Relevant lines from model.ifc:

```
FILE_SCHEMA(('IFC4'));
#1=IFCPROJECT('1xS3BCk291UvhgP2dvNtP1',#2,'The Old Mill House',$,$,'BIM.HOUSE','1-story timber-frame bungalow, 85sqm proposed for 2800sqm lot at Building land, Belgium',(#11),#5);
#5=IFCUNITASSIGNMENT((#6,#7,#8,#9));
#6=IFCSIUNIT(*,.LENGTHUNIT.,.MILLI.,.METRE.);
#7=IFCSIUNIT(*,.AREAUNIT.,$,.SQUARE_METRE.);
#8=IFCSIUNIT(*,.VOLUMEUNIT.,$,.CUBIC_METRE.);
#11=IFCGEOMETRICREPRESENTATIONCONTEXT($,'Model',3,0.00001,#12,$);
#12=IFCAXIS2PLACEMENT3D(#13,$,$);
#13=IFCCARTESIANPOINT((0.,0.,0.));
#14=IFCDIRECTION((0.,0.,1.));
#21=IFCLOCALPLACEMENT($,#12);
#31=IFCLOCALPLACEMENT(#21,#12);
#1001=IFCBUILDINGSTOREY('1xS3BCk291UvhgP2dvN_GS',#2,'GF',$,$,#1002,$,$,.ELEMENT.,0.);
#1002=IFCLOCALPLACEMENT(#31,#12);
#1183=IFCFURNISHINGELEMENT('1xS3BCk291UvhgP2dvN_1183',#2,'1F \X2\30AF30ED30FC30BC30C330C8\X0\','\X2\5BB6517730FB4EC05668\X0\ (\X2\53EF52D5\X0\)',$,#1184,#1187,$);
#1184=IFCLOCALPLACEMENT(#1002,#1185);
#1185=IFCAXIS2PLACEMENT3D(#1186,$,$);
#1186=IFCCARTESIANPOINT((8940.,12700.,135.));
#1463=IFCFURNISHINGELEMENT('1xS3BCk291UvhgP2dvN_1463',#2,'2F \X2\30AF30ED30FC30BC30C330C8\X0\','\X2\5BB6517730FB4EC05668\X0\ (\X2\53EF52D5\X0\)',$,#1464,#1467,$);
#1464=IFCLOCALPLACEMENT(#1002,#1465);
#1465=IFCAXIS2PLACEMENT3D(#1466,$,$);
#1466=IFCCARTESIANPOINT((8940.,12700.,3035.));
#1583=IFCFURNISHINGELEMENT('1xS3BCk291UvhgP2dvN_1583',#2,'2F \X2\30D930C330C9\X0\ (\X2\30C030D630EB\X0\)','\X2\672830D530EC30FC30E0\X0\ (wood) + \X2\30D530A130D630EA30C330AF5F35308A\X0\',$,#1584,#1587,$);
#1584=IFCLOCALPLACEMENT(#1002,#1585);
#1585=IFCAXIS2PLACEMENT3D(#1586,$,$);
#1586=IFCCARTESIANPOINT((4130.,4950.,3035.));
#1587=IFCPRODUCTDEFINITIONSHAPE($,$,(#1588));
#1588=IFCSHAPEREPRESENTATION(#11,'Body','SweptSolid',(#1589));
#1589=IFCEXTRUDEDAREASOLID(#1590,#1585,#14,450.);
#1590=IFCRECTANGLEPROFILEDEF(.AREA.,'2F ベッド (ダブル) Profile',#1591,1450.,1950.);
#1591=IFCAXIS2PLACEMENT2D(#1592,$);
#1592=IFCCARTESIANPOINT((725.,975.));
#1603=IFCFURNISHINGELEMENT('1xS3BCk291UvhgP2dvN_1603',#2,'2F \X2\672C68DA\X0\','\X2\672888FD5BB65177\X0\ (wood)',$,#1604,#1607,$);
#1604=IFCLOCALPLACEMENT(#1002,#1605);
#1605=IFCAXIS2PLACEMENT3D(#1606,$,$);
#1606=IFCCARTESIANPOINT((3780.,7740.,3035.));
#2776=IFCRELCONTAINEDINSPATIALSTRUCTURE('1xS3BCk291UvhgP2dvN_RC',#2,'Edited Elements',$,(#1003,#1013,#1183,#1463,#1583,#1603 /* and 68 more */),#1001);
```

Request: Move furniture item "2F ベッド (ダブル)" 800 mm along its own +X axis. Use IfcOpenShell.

```python
import ifcopenshell
import ifcopenshell.api.geometry
import ifcopenshell.util.placement

model = ifcopenshell.open("model.ifc")

item = model.by_id(1583)
matrix = ifcopenshell.util.placement.get_local_placement(item.ObjectPlacement)
matrix[:3, 3] += matrix[:3, 0] * 800.0
ifcopenshell.api.geometry.edit_object_placement(model, product=item, matrix=matrix, is_si=False)

print(ifcopenshell.util.placement.get_local_placement(item.ObjectPlacement).round(3) + 0.0)

model.write("model_updated.ifc")
```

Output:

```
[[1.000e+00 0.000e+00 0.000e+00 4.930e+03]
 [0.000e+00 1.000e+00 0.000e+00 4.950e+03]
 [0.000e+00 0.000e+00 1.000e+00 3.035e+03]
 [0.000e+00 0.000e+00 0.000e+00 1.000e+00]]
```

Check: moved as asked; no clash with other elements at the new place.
